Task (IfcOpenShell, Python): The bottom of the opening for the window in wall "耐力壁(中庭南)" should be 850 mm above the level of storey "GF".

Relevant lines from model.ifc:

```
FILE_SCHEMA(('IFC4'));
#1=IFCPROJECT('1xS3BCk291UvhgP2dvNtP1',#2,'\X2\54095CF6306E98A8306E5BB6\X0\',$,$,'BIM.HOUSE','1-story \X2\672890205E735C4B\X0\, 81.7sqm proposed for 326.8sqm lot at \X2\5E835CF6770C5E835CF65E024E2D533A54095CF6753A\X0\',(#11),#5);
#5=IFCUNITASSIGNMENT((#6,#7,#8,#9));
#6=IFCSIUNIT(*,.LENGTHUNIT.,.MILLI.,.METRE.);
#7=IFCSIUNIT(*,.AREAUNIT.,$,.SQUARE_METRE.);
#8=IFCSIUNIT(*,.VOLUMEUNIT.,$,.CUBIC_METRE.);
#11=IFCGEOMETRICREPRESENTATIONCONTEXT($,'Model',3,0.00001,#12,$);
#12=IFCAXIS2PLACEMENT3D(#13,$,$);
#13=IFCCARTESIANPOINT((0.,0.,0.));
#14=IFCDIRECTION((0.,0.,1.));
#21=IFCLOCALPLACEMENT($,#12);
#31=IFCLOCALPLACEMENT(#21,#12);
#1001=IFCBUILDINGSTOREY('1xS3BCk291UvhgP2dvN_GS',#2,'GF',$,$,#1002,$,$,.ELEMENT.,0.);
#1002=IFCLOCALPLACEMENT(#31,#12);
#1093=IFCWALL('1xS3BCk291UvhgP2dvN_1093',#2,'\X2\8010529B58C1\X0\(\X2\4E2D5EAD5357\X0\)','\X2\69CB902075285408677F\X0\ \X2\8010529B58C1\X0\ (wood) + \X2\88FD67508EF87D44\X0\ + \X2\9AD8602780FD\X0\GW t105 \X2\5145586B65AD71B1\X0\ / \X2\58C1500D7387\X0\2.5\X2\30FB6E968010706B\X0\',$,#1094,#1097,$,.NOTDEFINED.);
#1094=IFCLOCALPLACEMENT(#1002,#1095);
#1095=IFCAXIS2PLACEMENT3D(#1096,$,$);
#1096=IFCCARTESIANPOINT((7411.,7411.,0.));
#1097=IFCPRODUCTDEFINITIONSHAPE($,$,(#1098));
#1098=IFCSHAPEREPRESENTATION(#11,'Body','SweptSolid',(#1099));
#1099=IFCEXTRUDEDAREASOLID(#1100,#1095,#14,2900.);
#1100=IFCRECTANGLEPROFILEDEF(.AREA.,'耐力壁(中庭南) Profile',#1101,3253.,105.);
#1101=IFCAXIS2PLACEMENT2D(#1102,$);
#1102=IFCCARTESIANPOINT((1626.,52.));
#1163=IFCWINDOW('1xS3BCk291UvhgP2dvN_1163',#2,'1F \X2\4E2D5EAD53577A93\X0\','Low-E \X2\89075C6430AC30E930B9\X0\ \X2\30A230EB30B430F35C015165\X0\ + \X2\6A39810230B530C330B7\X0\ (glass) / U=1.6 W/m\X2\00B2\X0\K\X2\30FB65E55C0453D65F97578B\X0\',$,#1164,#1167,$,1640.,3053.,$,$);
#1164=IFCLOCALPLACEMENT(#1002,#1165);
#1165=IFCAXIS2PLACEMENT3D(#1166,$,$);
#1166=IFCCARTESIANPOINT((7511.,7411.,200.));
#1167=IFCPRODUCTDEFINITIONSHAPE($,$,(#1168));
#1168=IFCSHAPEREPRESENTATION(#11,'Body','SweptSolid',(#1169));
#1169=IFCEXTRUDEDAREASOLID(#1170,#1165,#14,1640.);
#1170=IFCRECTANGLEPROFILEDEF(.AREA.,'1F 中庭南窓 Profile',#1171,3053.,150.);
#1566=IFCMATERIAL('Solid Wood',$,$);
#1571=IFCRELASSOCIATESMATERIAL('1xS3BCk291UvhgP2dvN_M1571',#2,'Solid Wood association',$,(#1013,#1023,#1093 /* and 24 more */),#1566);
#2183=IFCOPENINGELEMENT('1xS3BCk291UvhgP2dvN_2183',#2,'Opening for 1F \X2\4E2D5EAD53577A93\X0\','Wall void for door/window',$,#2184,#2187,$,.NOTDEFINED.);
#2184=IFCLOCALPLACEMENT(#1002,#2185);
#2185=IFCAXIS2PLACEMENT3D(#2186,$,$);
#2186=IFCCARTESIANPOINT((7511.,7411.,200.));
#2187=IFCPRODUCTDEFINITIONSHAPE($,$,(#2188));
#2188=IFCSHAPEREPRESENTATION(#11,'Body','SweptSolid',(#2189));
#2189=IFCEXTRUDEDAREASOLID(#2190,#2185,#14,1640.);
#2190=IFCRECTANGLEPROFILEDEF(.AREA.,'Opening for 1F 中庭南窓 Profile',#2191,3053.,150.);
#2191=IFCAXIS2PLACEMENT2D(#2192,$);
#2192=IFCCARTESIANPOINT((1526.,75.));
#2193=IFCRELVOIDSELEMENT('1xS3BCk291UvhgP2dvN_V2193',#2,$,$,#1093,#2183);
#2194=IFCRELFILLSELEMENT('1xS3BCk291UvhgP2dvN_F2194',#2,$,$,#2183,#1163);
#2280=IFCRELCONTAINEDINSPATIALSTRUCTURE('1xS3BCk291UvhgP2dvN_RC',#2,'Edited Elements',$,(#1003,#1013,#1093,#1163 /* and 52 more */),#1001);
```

```python
import numpy as np
import ifcopenshell
import ifcopenshell.api.geometry
import ifcopenshell.geom
import ifcopenshell.util.element
import ifcopenshell.util.placement
import ifcopenshell.util.shape
import ifcopenshell.util.unit

model = ifcopenshell.open("model.ifc")
unit_scale = ifcopenshell.util.unit.calculate_unit_scale(model)

window = model.by_guid("1xS3BCk291UvhgP2dvN_1163")
opening = window.FillsVoids[0].RelatingOpeningElement
storey = ifcopenshell.util.element.get_container(window, ifc_class="IfcBuildingStorey")
level = ifcopenshell.util.placement.get_local_placement(storey.ObjectPlacement)[2, 3]

# The opening's origin need not be at the sill, so measure its lowest point.
shape = ifcopenshell.geom.create_shape(ifcopenshell.geom.settings(), opening)
bottom = ifcopenshell.util.shape.get_shape_bottom_elevation(shape, shape.geometry) / unit_scale
dz = level + 850.0 - bottom

shift = np.array([0.0, 0.0, dz])
# The window is not placed relative to its opening, so move both.
for product in (opening, window):
    matrix = ifcopenshell.util.placement.get_local_placement(product.ObjectPlacement)
    matrix[:3, 3] += shift
    ifcopenshell.api.geometry.edit_object_placement(model, product=product, matrix=matrix, is_si=False)

print(f"moved by {dz * unit_scale:+.3f} m")

model.write("model_v2.ifc")
```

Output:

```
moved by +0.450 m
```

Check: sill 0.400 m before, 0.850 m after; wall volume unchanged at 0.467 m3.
